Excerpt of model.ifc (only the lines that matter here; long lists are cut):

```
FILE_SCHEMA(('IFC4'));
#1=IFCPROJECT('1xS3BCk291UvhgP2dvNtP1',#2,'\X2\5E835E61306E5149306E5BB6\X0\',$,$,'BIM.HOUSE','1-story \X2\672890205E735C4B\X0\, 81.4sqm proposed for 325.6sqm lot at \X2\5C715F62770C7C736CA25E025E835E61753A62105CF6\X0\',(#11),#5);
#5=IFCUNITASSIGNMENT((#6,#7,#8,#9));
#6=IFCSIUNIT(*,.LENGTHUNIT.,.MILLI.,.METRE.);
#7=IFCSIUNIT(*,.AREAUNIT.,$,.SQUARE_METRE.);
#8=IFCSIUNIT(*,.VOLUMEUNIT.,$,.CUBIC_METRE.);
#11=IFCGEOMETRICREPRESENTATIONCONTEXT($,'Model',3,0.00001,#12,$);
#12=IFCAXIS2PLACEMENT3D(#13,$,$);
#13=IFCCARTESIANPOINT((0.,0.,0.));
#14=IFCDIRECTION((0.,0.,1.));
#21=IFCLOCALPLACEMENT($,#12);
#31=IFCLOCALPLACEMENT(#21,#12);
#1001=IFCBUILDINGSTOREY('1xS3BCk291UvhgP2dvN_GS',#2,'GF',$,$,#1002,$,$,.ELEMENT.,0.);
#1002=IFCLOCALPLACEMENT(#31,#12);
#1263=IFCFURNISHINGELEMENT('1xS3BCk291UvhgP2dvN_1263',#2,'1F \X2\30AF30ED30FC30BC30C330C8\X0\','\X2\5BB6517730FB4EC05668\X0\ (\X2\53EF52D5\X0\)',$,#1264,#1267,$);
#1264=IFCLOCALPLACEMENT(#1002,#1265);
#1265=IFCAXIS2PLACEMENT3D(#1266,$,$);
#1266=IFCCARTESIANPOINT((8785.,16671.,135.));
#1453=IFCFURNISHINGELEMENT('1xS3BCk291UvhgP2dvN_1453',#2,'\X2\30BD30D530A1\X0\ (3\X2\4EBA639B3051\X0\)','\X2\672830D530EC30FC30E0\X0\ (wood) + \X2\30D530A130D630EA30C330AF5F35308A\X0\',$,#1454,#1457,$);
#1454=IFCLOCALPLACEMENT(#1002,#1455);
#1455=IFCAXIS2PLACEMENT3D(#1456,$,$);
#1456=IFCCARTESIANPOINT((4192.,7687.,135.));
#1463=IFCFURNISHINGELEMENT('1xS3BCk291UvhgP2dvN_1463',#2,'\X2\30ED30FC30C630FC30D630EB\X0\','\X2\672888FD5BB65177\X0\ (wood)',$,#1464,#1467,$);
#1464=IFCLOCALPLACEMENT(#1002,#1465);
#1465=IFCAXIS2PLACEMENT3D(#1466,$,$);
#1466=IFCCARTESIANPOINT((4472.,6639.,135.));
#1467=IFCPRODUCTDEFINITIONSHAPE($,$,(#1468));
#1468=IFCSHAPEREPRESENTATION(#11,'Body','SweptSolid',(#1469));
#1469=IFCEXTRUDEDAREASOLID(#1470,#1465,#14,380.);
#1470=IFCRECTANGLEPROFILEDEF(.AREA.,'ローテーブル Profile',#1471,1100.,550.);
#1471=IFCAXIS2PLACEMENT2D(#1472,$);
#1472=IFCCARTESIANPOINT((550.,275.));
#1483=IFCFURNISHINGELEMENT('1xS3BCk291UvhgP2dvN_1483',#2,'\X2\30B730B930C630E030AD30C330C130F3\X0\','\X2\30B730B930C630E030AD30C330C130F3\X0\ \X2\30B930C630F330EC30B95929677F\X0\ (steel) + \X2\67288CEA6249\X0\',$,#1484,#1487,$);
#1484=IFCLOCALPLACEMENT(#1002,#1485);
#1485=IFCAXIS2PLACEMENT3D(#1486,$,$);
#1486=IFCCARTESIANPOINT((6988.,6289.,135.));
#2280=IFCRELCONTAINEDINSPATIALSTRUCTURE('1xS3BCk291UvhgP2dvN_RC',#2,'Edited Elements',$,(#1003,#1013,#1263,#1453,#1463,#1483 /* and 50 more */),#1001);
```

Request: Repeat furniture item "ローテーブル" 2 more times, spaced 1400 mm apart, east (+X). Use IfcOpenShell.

```python
import numpy as np
import ifcopenshell
import ifcopenshell.api.geometry
import ifcopenshell.api.root
import ifcopenshell.util.element
import ifcopenshell.util.placement

model = ifcopenshell.open("model.ifc")


def reuse_history(source, copy):
    """copy_class also copies each property set's owner history, people and application; keep the originals."""
    for rel in copy.IsDefinedBy:
        if rel.is_a("IfcRelDefinesByProperties") and (history := rel.RelatingPropertyDefinition.OwnerHistory):
            rel.RelatingPropertyDefinition.OwnerHistory = source.OwnerHistory
            ifcopenshell.util.element.remove_deep2(model, history)


source = model.by_guid("1xS3BCk291UvhgP2dvN_1463")
base = ifcopenshell.util.placement.get_local_placement(source.ObjectPlacement)
step = np.array([1.0, 0.0, 0.0]) * 1400.0

for i in range(1, 3):
    copy = ifcopenshell.api.root.copy_class(model, product=source)
    copy.Representation = ifcopenshell.util.element.copy_deep(
        model, source.Representation, exclude=["IfcGeometricRepresentationContext", "IfcRepresentationMap"]
    )
    reuse_history(source, copy)
    matrix = base.copy()
    matrix[:3, 3] += i * step
    print("added at", matrix[:3, 3].round(3) + 0.0)
    ifcopenshell.api.geometry.edit_object_placement(model, product=copy, matrix=matrix, is_si=False)

model.write("model_updated.ifc")
```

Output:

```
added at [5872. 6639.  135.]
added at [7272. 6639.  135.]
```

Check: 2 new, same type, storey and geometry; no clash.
